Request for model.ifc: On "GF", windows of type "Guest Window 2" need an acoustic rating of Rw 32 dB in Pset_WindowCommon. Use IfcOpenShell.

First a look at what the model holds.

```python
import ifcopenshell
import ifcopenshell.util.element

model = ifcopenshell.open("model.ifc")
print(model.schema)
storey = next(s for s in model.by_type("IfcBuildingStorey") if s.Name == "GF")
windows = [e for e in ifcopenshell.util.element.get_decomposition(storey) if e.is_a("IfcWindow")]
seen = {}
for e in windows:
    element_type = ifcopenshell.util.element.get_type(e)
    key = (element_type.Name if element_type != e and element_type else None, ifcopenshell.util.element.get_pset(e, "Pset_WindowCommon", "AcousticRating"))
    seen[key] = seen.get(key, 0) + 1
for (name, value), count in sorted(seen.items(), key=str):
    print(count, "x", name, "|", value)
```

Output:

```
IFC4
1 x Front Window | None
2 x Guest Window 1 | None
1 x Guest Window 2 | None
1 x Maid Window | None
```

```python
import ifcopenshell
import ifcopenshell.api.pset
import ifcopenshell.util.element

model = ifcopenshell.open("model.ifc")

storey = next(s for s in model.by_type("IfcBuildingStorey") if s.Name == "GF")
windows = [e for e in ifcopenshell.util.element.get_decomposition(storey) if e.is_a("IfcWindow")]

count = 0
for e in windows:
    element_type = ifcopenshell.util.element.get_type(e)
    if element_type in (None, e) or element_type.Name != "Guest Window 2":
        continue
    # add_pset returns the element's existing set when there is one.
    pset = ifcopenshell.api.pset.add_pset(model, product=e, name="Pset_WindowCommon")
    ifcopenshell.api.pset.edit_pset(model, pset=pset, properties={"AcousticRating": "Rw 32 dB"})
    count += 1

print(count, "windows updated")

model.write("model_v2.ifc")
```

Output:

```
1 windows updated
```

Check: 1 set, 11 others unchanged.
